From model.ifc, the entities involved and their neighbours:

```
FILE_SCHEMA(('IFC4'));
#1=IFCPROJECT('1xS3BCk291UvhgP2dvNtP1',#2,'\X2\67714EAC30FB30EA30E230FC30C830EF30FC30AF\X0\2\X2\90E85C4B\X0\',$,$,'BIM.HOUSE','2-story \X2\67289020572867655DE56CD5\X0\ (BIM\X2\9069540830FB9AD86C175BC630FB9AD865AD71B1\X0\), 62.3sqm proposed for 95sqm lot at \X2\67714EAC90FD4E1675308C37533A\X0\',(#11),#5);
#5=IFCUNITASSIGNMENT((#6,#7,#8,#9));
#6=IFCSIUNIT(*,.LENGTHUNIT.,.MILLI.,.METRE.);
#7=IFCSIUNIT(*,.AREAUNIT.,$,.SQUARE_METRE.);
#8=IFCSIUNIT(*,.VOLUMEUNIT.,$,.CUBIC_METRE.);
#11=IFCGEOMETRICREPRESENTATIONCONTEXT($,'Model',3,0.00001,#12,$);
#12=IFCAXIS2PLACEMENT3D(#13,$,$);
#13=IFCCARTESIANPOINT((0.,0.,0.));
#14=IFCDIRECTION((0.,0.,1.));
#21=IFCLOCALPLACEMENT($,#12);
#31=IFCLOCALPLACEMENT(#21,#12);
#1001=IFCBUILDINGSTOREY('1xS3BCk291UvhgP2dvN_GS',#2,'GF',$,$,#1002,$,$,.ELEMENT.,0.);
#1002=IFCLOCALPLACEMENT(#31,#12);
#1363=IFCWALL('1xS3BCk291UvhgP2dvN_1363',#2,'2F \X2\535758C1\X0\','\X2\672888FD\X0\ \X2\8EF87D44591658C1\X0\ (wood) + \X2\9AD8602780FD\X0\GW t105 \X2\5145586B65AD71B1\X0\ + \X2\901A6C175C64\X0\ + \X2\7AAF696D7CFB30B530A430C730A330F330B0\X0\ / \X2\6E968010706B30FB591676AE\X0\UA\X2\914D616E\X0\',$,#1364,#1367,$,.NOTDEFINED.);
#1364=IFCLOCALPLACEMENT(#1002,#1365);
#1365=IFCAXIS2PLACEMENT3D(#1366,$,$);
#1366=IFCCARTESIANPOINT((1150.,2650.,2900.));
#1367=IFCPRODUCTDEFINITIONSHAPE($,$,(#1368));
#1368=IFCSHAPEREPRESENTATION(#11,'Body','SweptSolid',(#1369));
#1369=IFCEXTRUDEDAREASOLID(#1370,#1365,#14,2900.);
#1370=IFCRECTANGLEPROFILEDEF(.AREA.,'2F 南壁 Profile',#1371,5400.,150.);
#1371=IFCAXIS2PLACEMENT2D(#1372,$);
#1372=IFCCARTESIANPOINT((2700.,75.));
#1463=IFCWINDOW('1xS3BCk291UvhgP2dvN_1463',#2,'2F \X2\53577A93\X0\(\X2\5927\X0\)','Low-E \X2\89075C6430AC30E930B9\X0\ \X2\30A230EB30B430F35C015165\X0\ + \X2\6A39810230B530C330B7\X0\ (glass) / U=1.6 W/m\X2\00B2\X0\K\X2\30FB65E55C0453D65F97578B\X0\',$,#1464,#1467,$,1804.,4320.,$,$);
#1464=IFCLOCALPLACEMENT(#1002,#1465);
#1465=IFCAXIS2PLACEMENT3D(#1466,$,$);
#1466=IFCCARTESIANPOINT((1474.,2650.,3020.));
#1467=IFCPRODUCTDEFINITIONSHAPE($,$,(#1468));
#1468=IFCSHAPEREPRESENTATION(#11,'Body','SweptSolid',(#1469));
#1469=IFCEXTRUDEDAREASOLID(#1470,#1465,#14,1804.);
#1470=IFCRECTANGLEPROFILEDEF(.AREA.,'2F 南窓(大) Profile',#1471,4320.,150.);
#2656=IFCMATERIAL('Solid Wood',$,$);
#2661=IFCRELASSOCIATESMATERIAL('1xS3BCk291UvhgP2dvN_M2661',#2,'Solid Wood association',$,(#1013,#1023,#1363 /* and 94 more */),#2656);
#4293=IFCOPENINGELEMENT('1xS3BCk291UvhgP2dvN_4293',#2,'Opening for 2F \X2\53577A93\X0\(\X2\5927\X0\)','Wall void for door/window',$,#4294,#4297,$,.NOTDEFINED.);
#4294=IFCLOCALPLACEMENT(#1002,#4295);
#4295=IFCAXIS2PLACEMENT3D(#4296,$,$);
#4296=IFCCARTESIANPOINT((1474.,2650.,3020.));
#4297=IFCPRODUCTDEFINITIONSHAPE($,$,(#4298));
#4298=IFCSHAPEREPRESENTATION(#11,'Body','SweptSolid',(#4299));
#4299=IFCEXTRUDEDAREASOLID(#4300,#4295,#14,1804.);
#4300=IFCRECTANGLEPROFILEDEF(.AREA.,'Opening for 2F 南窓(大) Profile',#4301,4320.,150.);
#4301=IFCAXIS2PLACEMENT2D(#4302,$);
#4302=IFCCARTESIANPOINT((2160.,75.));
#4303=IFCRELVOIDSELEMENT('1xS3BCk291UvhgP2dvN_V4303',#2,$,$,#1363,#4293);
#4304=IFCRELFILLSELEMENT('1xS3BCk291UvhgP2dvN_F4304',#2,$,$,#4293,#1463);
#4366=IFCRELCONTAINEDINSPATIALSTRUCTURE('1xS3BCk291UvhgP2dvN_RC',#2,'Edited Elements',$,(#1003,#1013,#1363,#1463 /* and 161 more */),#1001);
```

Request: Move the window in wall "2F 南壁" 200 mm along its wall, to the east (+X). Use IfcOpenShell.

```python
import ifcopenshell
import ifcopenshell.api.geometry
import ifcopenshell.util.placement
import ifcopenshell.util.unit

model = ifcopenshell.open("model.ifc")
unit_scale = ifcopenshell.util.unit.calculate_unit_scale(model)

window = model.by_id(1463)
opening = window.FillsVoids[0].RelatingOpeningElement
wall = opening.VoidsElements[0].RelatingBuildingElement

wall_matrix = ifcopenshell.util.placement.get_local_placement(wall.ObjectPlacement)
shift = wall_matrix[:3, 0] * 0.2 / unit_scale
before = ifcopenshell.util.placement.get_local_placement(window.ObjectPlacement)[:3, 3].copy()

# The window is not placed relative to its opening, so move both.
for product in (opening, window):
    matrix = ifcopenshell.util.placement.get_local_placement(product.ObjectPlacement)
    matrix[:3, 3] += shift
    ifcopenshell.api.geometry.edit_object_placement(model, product=product, matrix=matrix, is_si=False)

after = ifcopenshell.util.placement.get_local_placement(window.ObjectPlacement)[:3, 3]
print("window moved by", (after - before).round(3) + 0.0)

model.write("model_rev.ifc")
```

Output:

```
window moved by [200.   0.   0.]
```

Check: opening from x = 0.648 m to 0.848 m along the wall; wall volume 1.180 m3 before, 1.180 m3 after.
